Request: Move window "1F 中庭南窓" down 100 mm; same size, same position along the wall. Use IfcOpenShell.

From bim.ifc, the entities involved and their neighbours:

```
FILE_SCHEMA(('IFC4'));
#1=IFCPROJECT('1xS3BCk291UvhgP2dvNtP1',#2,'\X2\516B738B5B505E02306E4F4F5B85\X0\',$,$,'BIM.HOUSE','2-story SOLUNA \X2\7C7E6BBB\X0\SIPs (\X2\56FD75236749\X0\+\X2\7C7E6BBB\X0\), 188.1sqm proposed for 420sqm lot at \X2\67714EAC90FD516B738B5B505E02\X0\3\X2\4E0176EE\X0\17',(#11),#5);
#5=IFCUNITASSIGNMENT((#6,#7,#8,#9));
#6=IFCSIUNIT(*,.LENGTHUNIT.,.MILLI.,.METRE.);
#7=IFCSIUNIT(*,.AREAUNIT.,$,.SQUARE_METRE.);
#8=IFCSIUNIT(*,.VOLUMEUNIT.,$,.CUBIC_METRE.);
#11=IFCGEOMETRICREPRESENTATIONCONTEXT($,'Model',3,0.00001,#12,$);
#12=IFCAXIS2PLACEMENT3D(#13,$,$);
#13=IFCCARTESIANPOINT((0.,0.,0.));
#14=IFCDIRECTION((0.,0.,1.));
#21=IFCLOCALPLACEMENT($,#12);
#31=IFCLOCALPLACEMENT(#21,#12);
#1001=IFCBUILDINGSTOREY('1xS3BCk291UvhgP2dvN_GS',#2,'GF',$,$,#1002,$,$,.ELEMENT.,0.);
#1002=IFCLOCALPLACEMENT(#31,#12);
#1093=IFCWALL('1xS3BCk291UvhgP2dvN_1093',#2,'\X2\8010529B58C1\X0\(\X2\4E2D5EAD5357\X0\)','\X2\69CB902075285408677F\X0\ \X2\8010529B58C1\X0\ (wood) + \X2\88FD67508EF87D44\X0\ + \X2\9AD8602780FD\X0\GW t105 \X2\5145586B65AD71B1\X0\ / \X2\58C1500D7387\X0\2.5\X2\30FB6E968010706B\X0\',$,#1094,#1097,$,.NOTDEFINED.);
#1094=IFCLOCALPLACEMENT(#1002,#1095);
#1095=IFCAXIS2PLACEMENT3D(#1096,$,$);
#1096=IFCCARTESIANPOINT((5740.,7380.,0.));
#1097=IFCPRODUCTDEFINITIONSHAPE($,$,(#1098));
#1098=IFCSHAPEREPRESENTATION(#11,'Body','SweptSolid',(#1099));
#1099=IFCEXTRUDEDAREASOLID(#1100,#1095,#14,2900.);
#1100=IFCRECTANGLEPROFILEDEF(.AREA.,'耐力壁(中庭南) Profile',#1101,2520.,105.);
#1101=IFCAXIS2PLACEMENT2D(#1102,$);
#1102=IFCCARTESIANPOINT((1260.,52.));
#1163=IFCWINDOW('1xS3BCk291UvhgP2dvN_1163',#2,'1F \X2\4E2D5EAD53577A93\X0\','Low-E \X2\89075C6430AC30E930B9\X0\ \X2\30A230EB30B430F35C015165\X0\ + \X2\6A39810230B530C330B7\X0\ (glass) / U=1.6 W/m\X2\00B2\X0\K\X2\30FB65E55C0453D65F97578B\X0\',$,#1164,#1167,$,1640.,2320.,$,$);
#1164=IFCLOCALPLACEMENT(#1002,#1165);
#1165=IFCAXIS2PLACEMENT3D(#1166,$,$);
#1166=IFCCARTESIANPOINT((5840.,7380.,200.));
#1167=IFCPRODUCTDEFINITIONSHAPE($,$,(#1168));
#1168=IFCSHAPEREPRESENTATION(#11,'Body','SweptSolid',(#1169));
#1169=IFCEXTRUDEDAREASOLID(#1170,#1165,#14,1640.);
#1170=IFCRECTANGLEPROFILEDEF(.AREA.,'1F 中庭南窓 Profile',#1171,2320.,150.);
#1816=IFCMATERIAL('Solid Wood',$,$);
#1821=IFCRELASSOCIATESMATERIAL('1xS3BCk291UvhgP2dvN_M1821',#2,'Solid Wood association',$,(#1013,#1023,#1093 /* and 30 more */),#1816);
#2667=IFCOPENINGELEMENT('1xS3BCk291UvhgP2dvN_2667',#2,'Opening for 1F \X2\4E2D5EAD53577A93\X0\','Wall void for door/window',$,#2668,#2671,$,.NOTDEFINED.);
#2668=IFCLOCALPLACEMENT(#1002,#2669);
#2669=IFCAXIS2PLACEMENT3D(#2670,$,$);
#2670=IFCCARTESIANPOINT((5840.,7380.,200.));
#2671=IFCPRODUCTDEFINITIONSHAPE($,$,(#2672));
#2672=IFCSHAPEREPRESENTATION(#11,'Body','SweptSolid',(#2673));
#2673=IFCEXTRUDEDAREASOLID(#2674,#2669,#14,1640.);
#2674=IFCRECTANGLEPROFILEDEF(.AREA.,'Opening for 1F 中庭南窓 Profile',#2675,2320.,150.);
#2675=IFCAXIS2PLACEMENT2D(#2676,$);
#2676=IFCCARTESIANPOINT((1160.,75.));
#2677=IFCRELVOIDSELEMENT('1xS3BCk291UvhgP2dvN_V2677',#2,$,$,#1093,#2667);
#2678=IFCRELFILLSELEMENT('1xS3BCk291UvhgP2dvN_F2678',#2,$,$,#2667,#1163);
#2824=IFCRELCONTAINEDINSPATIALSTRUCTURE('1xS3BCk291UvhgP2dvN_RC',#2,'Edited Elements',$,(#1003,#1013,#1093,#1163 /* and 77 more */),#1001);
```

```python
import numpy as np
import ifcopenshell
import ifcopenshell.api.geometry
import ifcopenshell.util.placement
import ifcopenshell.util.unit

model = ifcopenshell.open("bim.ifc")
unit_scale = ifcopenshell.util.unit.calculate_unit_scale(model)

window = model.by_id(1163)
opening = window.FillsVoids[0].RelatingOpeningElement
dz = -0.1 / unit_scale

shift = np.array([0.0, 0.0, dz])
# The window is not placed relative to its opening, so move both.
for product in (opening, window):
    matrix = ifcopenshell.util.placement.get_local_placement(product.ObjectPlacement)
    matrix[:3, 3] += shift
    ifcopenshell.api.geometry.edit_object_placement(model, product=product, matrix=matrix, is_si=False)

print(f"moved by {dz * unit_scale:+.3f} m")

model.write("bim_edited.ifc")
```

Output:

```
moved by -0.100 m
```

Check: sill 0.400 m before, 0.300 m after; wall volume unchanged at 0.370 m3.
